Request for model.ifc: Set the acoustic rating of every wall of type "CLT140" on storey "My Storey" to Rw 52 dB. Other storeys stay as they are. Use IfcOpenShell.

First a look at what the model holds.

```python
import ifcopenshell
import ifcopenshell.util.element

model = ifcopenshell.open("model.ifc")
print(model.schema)
storey = next(s for s in model.by_type("IfcBuildingStorey") if s.Name == "My Storey")
walls = [e for e in ifcopenshell.util.element.get_decomposition(storey) if e.is_a("IfcWall")]
seen = {}
for e in walls:
    element_type = ifcopenshell.util.element.get_type(e)
    key = (element_type.Name if element_type != e and element_type else None, ifcopenshell.util.element.get_pset(e, "Pset_WallCommon", "AcousticRating"))
    seen[key] = seen.get(key, 0) + 1
for (name, value), count in sorted(seen.items(), key=str):
    print(count, "x", name, "|", value)
```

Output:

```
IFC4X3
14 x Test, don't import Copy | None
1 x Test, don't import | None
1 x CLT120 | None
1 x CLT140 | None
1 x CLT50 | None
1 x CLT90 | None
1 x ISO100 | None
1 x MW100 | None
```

```python
import ifcopenshell
import ifcopenshell.api.pset
import ifcopenshell.util.element

model = ifcopenshell.open("model.ifc")

storey = next(s for s in model.by_type("IfcBuildingStorey") if s.Name == "My Storey")
walls = [e for e in ifcopenshell.util.element.get_decomposition(storey) if e.is_a("IfcWall")]

count = 0
for e in walls:
    element_type = ifcopenshell.util.element.get_type(e)
    if element_type in (None, e) or element_type.Name != "CLT140":
        continue
    # add_pset returns the element's existing set when there is one.
    pset = ifcopenshell.api.pset.add_pset(model, product=e, name="Pset_WallCommon")
    ifcopenshell.api.pset.edit_pset(model, pset=pset, properties={"AcousticRating": "Rw 52 dB"})
    count += 1

print(count, "walls updated")

model.write("model_updated.ifc")
```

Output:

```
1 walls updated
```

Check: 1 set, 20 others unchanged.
